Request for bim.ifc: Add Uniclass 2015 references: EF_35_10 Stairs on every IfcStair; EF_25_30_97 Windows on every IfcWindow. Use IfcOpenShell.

First a look at what the model holds.

```python
import ifcopenshell

model = ifcopenshell.open("bim.ifc")
print(model.schema)
print("classifications:", [c.Name for c in model.by_type("IfcClassification")])
for ifc_class in ("IfcDoor", "IfcRoof", "IfcStair", "IfcWall", "IfcWindow"):
    print(ifc_class, len(model.by_type(ifc_class)))
```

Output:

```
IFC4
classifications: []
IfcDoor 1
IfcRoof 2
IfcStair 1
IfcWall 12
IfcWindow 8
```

```python
import ifcopenshell
import ifcopenshell.api.classification

model = ifcopenshell.open("bim.ifc")

system = ifcopenshell.api.classification.add_classification(model, classification="Uniclass 2015")

codes = {
    "IfcStair": ("EF_35_10", "Stairs"),
    "IfcWindow": ("EF_25_30_97", "Windows"),
}
for ifc_class, (code, name) in codes.items():
    products = model.by_type(ifc_class)
    ifcopenshell.api.classification.add_reference(
        model, products=products, classification=system, identification=code, name=name
    )
    print(code, len(products))

model.write("bim_rev.ifc")
```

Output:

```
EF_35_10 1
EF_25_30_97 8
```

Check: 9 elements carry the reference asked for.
